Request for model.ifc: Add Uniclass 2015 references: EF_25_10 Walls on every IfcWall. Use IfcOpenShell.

First a look at what the model holds.

```python
import ifcopenshell

model = ifcopenshell.open("model.ifc")
print(model.schema)
print("classifications:", [c.Name for c in model.by_type("IfcClassification")])
for ifc_class in ("IfcDoor", "IfcRoof", "IfcStair", "IfcWall", "IfcWindow"):
    print(ifc_class, len(model.by_type(ifc_class)))
```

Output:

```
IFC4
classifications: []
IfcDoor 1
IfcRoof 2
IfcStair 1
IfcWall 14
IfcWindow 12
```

```python
import ifcopenshell
import ifcopenshell.api.classification

model = ifcopenshell.open("model.ifc")

system = ifcopenshell.api.classification.add_classification(model, classification="Uniclass 2015")

codes = {
    "IfcWall": ("EF_25_10", "Walls"),
}
for ifc_class, (code, name) in codes.items():
    products = model.by_type(ifc_class)
    ifcopenshell.api.classification.add_reference(
        model, products=products, classification=system, identification=code, name=name
    )
    print(code, len(products))

model.write("model_rev.ifc")
```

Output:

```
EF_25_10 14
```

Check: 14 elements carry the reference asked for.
